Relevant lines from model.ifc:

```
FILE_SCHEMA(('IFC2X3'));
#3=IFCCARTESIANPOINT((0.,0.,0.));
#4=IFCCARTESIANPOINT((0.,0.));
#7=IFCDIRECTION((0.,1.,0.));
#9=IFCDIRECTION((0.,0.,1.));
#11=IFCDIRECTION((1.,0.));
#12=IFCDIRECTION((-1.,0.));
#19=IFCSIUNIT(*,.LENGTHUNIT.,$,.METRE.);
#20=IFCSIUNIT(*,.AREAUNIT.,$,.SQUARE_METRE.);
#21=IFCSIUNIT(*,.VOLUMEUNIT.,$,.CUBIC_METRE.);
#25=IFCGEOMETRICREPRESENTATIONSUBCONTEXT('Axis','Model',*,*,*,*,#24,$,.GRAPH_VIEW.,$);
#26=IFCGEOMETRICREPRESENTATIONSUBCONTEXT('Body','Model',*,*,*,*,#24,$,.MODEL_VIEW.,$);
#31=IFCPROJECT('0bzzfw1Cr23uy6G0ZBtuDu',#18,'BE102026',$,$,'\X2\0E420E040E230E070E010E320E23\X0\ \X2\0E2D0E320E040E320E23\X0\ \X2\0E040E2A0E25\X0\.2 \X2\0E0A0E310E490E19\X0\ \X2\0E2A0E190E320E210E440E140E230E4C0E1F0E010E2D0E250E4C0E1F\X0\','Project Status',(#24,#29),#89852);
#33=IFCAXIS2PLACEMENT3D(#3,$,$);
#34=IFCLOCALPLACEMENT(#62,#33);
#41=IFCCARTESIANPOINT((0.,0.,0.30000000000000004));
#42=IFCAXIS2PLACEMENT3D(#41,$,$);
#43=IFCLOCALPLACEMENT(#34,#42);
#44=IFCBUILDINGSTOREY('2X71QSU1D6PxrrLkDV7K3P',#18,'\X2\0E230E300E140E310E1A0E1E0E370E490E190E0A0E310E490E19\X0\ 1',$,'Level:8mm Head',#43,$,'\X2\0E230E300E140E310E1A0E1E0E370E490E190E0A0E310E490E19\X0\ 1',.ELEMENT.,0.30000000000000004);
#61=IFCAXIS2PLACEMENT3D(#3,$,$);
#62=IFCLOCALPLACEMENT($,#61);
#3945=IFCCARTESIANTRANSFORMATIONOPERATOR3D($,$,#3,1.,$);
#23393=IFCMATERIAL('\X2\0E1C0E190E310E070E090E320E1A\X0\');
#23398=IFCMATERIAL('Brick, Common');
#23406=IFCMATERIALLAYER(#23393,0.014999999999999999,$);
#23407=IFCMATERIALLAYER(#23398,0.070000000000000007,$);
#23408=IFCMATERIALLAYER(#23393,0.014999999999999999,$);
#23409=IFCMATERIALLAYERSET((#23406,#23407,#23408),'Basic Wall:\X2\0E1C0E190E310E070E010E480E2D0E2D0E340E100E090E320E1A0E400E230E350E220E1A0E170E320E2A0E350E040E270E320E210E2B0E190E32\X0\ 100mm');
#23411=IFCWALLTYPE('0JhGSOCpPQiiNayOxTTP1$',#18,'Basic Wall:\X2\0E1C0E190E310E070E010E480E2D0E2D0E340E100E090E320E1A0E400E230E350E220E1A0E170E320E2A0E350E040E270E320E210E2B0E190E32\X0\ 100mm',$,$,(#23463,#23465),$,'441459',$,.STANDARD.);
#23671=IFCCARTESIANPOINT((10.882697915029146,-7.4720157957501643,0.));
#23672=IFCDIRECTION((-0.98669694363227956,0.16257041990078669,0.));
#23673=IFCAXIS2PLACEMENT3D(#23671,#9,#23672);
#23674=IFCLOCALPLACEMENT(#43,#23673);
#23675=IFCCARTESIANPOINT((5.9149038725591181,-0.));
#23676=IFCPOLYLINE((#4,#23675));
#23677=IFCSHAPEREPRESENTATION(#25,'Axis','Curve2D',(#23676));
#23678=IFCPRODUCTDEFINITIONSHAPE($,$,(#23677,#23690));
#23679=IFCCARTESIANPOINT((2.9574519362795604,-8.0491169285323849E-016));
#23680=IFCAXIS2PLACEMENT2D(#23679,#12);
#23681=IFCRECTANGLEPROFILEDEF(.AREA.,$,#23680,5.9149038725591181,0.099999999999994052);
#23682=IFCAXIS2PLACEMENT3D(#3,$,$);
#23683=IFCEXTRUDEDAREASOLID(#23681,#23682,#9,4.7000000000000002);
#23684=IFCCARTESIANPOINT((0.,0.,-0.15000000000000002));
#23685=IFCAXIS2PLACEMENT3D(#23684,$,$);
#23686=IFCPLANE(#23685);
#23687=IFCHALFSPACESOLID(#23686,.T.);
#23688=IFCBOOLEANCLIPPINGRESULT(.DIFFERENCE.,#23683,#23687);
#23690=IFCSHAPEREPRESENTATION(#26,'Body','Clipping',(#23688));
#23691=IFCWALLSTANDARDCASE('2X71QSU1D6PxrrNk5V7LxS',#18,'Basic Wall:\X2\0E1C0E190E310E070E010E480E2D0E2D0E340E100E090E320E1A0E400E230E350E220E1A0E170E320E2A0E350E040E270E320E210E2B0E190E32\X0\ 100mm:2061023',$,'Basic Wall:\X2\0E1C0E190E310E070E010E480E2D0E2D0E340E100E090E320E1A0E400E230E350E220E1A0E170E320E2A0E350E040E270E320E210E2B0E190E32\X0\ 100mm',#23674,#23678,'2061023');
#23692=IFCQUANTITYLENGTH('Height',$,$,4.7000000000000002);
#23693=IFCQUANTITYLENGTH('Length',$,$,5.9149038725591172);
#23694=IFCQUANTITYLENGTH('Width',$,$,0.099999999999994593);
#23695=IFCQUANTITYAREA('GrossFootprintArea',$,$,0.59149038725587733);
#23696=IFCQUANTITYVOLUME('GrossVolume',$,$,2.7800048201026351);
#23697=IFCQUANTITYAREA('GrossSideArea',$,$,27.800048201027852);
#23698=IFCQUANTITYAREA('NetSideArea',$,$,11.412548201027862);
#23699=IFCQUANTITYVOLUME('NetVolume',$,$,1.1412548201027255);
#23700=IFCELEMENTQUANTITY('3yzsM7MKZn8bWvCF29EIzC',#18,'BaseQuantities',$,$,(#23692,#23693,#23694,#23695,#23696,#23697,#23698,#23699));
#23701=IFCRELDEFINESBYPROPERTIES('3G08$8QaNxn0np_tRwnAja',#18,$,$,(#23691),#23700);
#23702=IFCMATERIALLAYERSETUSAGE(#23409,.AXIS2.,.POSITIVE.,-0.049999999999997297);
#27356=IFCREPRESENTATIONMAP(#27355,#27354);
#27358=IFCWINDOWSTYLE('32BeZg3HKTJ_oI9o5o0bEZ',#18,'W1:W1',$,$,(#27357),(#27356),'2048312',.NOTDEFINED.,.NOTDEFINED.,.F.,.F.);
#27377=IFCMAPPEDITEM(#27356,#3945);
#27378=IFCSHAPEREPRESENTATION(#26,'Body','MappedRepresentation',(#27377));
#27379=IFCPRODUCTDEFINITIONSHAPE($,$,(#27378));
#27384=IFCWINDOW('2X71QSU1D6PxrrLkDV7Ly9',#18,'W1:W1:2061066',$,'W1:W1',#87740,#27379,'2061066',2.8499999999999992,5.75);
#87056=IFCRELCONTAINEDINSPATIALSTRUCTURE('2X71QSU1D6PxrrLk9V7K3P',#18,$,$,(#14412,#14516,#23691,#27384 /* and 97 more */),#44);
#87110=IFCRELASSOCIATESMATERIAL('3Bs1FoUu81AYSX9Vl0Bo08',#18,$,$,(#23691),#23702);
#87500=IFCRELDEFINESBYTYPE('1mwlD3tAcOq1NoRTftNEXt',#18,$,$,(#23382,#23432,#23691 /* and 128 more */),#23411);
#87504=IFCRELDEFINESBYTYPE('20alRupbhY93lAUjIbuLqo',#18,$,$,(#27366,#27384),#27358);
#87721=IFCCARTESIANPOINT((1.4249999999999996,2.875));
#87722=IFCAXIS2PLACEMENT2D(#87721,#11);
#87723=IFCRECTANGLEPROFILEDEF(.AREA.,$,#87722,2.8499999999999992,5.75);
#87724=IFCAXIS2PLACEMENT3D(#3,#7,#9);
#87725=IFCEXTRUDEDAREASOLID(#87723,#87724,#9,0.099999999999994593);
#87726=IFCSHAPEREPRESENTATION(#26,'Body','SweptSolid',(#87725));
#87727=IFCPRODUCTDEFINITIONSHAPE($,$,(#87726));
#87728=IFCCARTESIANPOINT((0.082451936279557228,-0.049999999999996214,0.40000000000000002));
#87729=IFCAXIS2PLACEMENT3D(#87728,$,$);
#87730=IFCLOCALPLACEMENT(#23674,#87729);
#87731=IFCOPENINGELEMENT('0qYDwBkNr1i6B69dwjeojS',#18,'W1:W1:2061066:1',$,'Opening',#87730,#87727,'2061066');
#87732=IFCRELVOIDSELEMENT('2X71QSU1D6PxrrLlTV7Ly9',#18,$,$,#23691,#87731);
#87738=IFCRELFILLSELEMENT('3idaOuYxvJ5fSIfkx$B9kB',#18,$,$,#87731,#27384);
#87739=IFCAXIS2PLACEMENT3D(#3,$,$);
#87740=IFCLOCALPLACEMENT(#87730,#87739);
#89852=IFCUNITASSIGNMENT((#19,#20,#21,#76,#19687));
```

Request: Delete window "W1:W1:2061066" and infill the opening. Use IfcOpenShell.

```python
import ifcopenshell
import ifcopenshell.api.feature
import ifcopenshell.api.pset
import ifcopenshell.api.root
import ifcopenshell.geom
import ifcopenshell.util.element
import ifcopenshell.util.shape
import ifcopenshell.util.unit

model = ifcopenshell.open("model.ifc")
area_scale = ifcopenshell.util.unit.calculate_unit_scale(model, "AREAUNIT")
volume_scale = ifcopenshell.util.unit.calculate_unit_scale(model, "VOLUMEUNIT")
settings = ifcopenshell.geom.settings()


def volume(element):
    """Net volume in cubic metres, openings subtracted."""
    shape = ifcopenshell.geom.create_shape(settings, element)
    return ifcopenshell.util.shape.get_volume(shape.geometry)


window = model.by_guid("2X71QSU1D6PxrrLkDV7Ly9")
opening = window.FillsVoids[0].RelatingOpeningElement
wall = opening.VoidsElements[0].RelatingBuildingElement
before = volume(wall)

ifcopenshell.api.root.remove_product(model, product=window)
ifcopenshell.api.feature.remove_feature(model, feature=opening)

after = volume(wall)
thickness = 0.1  # wall thickness in metres

# Update the wall's stored quantities.
qto = model.by_id(ifcopenshell.util.element.get_pset(wall, "BaseQuantities", should_inherit=False)["id"])
ifcopenshell.api.pset.edit_qto(model, qto=qto, properties={
    "NetSideArea": after / thickness / area_scale,
    "NetVolume": after / volume_scale,
})

print(f"wall volume {before:.3f} -> {after:.3f} m3")

model.write("model-out.ifc")
```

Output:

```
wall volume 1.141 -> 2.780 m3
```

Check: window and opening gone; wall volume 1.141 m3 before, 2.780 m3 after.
